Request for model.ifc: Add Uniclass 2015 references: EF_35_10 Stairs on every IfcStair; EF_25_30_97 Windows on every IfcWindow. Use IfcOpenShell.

First a look at what the model holds.

```python
import ifcopenshell

model = ifcopenshell.open("model.ifc")
print(model.schema)
print("classifications:", [c.Name for c in model.by_type("IfcClassification")])
for ifc_class in ("IfcDoor", "IfcRoof", "IfcStair", "IfcWall", "IfcWindow"):
    print(ifc_class, len(model.by_type(ifc_class)))
```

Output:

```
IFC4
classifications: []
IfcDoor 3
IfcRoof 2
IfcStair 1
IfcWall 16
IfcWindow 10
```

```python
import ifcopenshell
import ifcopenshell.api.classification

model = ifcopenshell.open("model.ifc")

system = ifcopenshell.api.classification.add_classification(model, classification="Uniclass 2015")

codes = {
    "IfcStair": ("EF_35_10", "Stairs"),
    "IfcWindow": ("EF_25_30_97", "Windows"),
}
for ifc_class, (code, name) in codes.items():
    products = model.by_type(ifc_class)
    ifcopenshell.api.classification.add_reference(
        model, products=products, classification=system, identification=code, name=name
    )
    print(code, len(products))

model.write("model_v2.ifc")
```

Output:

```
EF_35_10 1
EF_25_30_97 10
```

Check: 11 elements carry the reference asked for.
